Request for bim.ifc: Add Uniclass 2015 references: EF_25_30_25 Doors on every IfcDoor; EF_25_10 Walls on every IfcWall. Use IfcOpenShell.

First a look at what the model holds.

```python
import ifcopenshell

model = ifcopenshell.open("bim.ifc")
print(model.schema)
print("classifications:", [c.Name for c in model.by_type("IfcClassification")])
for ifc_class in ("IfcDoor", "IfcRoof", "IfcStair", "IfcWall", "IfcWindow"):
    print(ifc_class, len(model.by_type(ifc_class)))
```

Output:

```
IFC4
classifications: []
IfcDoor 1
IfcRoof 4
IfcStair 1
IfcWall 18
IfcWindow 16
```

```python
import ifcopenshell
import ifcopenshell.api.classification

model = ifcopenshell.open("bim.ifc")

system = ifcopenshell.api.classification.add_classification(model, classification="Uniclass 2015")

codes = {
    "IfcDoor": ("EF_25_30_25", "Doors"),
    "IfcWall": ("EF_25_10", "Walls"),
}
for ifc_class, (code, name) in codes.items():
    products = model.by_type(ifc_class)
    ifcopenshell.api.classification.add_reference(
        model, products=products, classification=system, identification=code, name=name
    )
    print(code, len(products))

model.write("bim-out.ifc")
```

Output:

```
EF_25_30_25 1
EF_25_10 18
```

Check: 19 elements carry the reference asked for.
